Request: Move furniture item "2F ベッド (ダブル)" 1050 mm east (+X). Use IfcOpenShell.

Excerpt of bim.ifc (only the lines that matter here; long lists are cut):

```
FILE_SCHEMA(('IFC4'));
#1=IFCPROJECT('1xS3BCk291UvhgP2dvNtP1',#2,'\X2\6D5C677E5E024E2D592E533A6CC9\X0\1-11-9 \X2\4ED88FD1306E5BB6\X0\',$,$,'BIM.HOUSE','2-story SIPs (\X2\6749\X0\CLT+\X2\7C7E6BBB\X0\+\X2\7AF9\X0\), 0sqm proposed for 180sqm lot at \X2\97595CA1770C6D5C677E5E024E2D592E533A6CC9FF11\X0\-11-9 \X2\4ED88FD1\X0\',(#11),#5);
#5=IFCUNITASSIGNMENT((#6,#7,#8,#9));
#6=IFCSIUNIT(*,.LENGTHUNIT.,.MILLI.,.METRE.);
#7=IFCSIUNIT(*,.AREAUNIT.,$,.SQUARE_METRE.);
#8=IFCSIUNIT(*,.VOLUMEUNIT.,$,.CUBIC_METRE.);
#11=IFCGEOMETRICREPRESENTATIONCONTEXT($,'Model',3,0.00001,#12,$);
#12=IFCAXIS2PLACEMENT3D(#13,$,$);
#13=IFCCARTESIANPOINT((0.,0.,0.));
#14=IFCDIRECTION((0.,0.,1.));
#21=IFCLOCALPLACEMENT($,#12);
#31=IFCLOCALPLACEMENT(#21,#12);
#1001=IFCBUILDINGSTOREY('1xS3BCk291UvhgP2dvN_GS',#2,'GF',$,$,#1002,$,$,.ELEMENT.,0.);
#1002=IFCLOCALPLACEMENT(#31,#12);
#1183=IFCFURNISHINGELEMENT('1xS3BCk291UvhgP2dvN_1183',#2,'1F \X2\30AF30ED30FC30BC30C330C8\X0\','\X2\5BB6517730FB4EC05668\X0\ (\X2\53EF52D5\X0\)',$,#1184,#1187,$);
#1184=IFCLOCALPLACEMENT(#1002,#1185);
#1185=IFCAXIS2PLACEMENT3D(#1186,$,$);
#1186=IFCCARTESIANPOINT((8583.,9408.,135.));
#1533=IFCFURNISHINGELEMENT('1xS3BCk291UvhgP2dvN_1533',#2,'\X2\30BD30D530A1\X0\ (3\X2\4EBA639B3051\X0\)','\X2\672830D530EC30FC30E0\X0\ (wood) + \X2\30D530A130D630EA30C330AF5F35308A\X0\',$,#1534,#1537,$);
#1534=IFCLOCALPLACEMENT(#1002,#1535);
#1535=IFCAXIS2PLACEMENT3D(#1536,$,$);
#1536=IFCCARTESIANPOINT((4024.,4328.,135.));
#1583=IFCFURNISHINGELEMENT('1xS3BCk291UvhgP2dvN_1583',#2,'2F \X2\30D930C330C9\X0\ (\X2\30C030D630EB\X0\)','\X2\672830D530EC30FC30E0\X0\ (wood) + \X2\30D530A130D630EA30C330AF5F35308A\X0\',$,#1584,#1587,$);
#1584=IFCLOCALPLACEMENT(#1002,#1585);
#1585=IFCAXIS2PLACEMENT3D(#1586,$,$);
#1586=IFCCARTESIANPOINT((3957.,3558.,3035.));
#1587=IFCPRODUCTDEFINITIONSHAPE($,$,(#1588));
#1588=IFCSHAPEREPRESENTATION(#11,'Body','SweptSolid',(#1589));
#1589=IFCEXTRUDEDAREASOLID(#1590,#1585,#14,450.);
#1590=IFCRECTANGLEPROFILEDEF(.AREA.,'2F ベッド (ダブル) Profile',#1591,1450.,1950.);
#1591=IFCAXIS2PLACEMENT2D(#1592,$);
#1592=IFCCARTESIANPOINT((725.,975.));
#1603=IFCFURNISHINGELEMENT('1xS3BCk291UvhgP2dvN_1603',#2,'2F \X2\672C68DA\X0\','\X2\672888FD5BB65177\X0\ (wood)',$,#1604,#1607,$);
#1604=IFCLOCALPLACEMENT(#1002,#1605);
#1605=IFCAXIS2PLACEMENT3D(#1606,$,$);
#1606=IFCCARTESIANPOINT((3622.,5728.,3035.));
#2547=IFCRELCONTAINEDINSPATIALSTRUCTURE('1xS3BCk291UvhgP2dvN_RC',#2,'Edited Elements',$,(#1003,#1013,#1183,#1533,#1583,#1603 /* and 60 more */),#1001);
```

```python
import ifcopenshell
import ifcopenshell.api.geometry
import ifcopenshell.util.placement
import ifcopenshell.util.unit

model = ifcopenshell.open("bim.ifc")
unit_scale = ifcopenshell.util.unit.calculate_unit_scale(model)

item = model.by_guid("1xS3BCk291UvhgP2dvN_1583")
matrix = ifcopenshell.util.placement.get_local_placement(item.ObjectPlacement)
matrix[0, 3] += 1.05 / unit_scale
ifcopenshell.api.geometry.edit_object_placement(model, product=item, matrix=matrix, is_si=False)

print(ifcopenshell.util.placement.get_local_placement(item.ObjectPlacement).round(3) + 0.0)

model.write("bim_updated.ifc")
```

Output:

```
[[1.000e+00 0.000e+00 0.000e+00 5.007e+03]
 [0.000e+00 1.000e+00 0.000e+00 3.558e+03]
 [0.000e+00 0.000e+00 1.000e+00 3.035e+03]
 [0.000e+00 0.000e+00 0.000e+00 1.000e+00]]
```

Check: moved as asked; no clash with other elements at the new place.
